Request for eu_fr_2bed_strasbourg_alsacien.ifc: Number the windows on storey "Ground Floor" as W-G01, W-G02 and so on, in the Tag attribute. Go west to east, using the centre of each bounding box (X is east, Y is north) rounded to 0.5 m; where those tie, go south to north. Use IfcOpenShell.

First a look at what the model holds.

```python
import ifcopenshell
import ifcopenshell.util.element
import ifcopenshell.util.placement

model = ifcopenshell.open("eu_fr_2bed_strasbourg_alsacien.ifc")
print(model.schema)
storey = next(s for s in model.by_type("IfcBuildingStorey") if s.Name == "Ground Floor")
windows = [e for e in ifcopenshell.util.element.get_decomposition(storey) if e.is_a("IfcWindow")]
for e in sorted(windows, key=lambda e: e.id()):
    origin = ifcopenshell.util.placement.get_local_placement(e.ObjectPlacement)[:3, 3]
    print(e.id(), e.Tag, e.Name, origin.round(2) + 0.0, sep=" | ")
```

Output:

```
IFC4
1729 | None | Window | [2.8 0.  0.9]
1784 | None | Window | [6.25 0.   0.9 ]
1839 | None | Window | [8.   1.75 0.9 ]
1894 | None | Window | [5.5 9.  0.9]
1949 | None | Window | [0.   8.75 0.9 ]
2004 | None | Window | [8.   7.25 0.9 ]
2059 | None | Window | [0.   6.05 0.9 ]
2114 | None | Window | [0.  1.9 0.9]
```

```python
import ifcopenshell
import ifcopenshell.geom
import ifcopenshell.util.element
import ifcopenshell.util.shape

model = ifcopenshell.open("eu_fr_2bed_strasbourg_alsacien.ifc")
settings = ifcopenshell.geom.settings()
settings.set("use-world-coords", True)


def centre(element):
    shape = ifcopenshell.geom.create_shape(settings, element)
    return ifcopenshell.util.shape.get_bbox_centroid(shape.geometry)


storey = next(s for s in model.by_type("IfcBuildingStorey") if s.Name == "Ground Floor")
windows = [e for e in ifcopenshell.util.element.get_decomposition(storey) if e.is_a("IfcWindow")]

# Insertion points can sit at a corner or the storey origin, so sort by the geometry (in metres).
centres = {e: centre(e) for e in windows}
windows.sort(key=lambda e: (round(centres[e][0] / 0.5), centres[e][1]))

for i, e in enumerate(windows, start=1):
    number = f"W-G{i:02d}"
    e.Tag = number
    print(e.id(), number)

model.write("eu_fr_2bed_strasbourg_alsacien_rev.ifc")
```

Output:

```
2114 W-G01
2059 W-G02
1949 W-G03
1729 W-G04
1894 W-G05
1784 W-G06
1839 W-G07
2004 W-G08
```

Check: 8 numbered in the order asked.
